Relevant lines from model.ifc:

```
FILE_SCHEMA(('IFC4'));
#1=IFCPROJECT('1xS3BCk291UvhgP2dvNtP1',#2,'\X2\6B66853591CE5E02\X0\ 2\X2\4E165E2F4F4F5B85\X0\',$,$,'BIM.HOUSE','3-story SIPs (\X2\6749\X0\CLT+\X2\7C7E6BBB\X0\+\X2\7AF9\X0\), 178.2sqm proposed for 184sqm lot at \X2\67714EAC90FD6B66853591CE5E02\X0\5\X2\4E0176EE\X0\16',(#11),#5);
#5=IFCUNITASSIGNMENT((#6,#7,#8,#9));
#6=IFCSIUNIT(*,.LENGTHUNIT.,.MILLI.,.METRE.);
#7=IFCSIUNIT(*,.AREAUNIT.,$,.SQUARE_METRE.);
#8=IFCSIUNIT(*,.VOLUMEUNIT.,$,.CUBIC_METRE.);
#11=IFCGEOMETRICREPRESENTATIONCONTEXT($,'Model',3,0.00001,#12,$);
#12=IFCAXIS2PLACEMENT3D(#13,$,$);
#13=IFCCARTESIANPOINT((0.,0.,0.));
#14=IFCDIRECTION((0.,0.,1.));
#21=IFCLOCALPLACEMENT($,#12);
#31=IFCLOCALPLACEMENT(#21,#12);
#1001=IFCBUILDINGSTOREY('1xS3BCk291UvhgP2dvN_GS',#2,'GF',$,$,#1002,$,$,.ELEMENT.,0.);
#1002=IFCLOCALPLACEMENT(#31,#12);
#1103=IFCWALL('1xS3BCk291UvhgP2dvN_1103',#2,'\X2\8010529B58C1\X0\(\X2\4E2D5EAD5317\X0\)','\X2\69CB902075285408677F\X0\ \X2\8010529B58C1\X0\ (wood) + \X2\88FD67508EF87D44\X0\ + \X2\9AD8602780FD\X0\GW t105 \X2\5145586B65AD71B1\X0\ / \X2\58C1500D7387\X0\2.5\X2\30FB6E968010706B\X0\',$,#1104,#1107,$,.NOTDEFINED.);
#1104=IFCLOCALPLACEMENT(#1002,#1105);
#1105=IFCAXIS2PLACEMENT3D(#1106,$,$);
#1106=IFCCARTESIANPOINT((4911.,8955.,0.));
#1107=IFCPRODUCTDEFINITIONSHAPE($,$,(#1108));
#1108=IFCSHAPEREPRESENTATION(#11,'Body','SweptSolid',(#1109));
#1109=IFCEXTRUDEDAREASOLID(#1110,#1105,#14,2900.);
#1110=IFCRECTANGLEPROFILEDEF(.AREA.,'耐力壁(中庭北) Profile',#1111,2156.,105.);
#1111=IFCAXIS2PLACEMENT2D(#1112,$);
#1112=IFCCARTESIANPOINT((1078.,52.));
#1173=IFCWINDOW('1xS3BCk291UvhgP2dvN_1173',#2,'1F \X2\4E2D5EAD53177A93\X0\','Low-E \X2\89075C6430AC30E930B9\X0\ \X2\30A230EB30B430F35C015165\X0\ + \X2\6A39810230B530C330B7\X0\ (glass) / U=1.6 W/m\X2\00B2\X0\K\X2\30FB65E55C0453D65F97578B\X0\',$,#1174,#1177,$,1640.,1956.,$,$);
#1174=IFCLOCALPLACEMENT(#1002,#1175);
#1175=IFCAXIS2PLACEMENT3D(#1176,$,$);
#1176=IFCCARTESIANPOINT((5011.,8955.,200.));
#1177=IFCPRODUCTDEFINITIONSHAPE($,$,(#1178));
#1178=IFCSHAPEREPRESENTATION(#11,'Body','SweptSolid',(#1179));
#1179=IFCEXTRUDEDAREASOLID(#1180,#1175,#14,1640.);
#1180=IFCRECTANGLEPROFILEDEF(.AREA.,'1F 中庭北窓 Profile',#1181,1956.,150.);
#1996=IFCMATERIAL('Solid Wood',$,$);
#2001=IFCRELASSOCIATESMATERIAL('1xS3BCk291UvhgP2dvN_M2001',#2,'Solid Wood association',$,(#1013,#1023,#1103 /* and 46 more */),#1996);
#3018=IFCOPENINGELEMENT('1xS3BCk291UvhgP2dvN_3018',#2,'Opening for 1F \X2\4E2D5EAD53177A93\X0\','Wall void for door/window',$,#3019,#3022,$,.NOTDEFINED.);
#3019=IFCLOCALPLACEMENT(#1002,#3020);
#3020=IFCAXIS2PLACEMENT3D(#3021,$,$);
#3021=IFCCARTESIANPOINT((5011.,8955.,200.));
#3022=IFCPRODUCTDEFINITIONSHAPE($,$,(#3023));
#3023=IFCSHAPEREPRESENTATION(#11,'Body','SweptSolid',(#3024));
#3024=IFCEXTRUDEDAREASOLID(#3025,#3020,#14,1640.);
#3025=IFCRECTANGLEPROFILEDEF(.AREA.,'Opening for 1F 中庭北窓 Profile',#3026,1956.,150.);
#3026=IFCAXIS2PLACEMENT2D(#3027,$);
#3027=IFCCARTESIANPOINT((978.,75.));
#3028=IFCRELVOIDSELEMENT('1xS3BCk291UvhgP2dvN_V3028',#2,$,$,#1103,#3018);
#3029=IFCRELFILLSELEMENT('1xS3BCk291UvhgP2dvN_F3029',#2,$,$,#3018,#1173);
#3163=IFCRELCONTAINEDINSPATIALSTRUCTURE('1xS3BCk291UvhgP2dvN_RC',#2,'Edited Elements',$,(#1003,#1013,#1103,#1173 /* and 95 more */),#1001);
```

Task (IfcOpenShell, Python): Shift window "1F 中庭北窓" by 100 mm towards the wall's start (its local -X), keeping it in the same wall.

```python
import ifcopenshell
import ifcopenshell.api.geometry
import ifcopenshell.util.placement

model = ifcopenshell.open("model.ifc")

window = model.by_id(1173)
opening = window.FillsVoids[0].RelatingOpeningElement
wall = opening.VoidsElements[0].RelatingBuildingElement

wall_matrix = ifcopenshell.util.placement.get_local_placement(wall.ObjectPlacement)
shift = wall_matrix[:3, 0] * -100.0
before = ifcopenshell.util.placement.get_local_placement(window.ObjectPlacement)[:3, 3].copy()

# The window is not placed relative to its opening, so move both.
for product in (opening, window):
    matrix = ifcopenshell.util.placement.get_local_placement(product.ObjectPlacement)
    matrix[:3, 3] += shift
    ifcopenshell.api.geometry.edit_object_placement(model, product=product, matrix=matrix, is_si=False)

after = ifcopenshell.util.placement.get_local_placement(window.ObjectPlacement)[:3, 3]
print("window moved by", (after - before).round(3) + 0.0)

model.write("model_rev.ifc")
```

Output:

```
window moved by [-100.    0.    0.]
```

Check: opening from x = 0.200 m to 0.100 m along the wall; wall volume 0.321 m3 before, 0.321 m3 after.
